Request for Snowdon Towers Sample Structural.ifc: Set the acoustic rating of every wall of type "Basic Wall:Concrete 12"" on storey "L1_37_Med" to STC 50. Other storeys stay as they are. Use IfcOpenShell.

First a look at what the model holds.

```python
import ifcopenshell
import ifcopenshell.util.element

model = ifcopenshell.open("Snowdon Towers Sample Structural.ifc")
print(model.schema)
storey = next(s for s in model.by_type("IfcBuildingStorey") if s.Name == "L1_37_Med")
walls = [e for e in ifcopenshell.util.element.get_decomposition(storey) if e.is_a("IfcWall")]
seen = {}
for e in walls:
    element_type = ifcopenshell.util.element.get_type(e)
    key = (element_type.Name if element_type != e and element_type else None, ifcopenshell.util.element.get_pset(e, "Pset_WallCommon", "AcousticRating"))
    seen[key] = seen.get(key, 0) + 1
for (name, value), count in sorted(seen.items(), key=str):
    print(count, "x", name, "|", value)
```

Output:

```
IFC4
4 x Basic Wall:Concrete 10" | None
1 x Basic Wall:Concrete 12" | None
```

```python
import ifcopenshell
import ifcopenshell.api.pset
import ifcopenshell.util.element

model = ifcopenshell.open("Snowdon Towers Sample Structural.ifc")

storey = next(s for s in model.by_type("IfcBuildingStorey") if s.Name == "L1_37_Med")
walls = [e for e in ifcopenshell.util.element.get_decomposition(storey) if e.is_a("IfcWall")]

count = 0
for e in walls:
    element_type = ifcopenshell.util.element.get_type(e)
    if element_type in (None, e) or element_type.Name != 'Basic Wall:Concrete 12"':
        continue
    # add_pset returns the element's existing set when there is one.
    pset = ifcopenshell.api.pset.add_pset(model, product=e, name="Pset_WallCommon")
    ifcopenshell.api.pset.edit_pset(model, pset=pset, properties={"AcousticRating": "STC 50"})
    count += 1

print(count, "walls updated")

model.write("Snowdon Towers Sample Structural_updated.ifc")
```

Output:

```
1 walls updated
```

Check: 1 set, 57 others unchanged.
